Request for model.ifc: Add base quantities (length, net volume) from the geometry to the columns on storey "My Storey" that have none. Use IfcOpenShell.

First a look at what the model holds.

```python
import ifcopenshell
import ifcopenshell.util.element
import ifcopenshell.util.unit

model = ifcopenshell.open("model.ifc")
print(model.schema)
for unit_type in ("LENGTHUNIT", "AREAUNIT", "VOLUMEUNIT"):
    print(unit_type, ifcopenshell.util.unit.calculate_unit_scale(model, unit_type))
storey = next(s for s in model.by_type("IfcBuildingStorey") if s.Name == "My Storey")
columns = [e for e in ifcopenshell.util.element.get_decomposition(storey) if e.is_a("IfcColumn")]
for e in sorted(columns, key=lambda e: e.id()):
    print(e.id(), e.is_a(), e.Name, list(ifcopenshell.util.element.get_psets(e, qtos_only=True)), sep=" | ")
```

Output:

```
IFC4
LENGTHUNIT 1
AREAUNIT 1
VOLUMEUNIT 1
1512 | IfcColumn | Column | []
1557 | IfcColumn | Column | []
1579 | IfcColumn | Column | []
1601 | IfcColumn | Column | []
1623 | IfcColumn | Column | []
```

```python
import ifcopenshell
import ifcopenshell.api.pset
import ifcopenshell.geom
import ifcopenshell.util.element
import ifcopenshell.util.shape
import ifcopenshell.util.unit

model = ifcopenshell.open("model.ifc")
unit_scale = ifcopenshell.util.unit.calculate_unit_scale(model)
volume_scale = ifcopenshell.util.unit.calculate_unit_scale(model, "VOLUMEUNIT")
settings = ifcopenshell.geom.settings()

storey = next(s for s in model.by_type("IfcBuildingStorey") if s.Name == "My Storey")
columns = [e for e in ifcopenshell.util.element.get_decomposition(storey) if e.is_a("IfcColumn")]

for e in sorted(columns, key=lambda e: e.id()):
    if ifcopenshell.util.element.get_psets(e, qtos_only=True, should_inherit=False):
        continue
    # Geometry comes back in metres, in the element's own axes.
    shape = ifcopenshell.geom.create_shape(settings, e)
    values = {
        "Length": ifcopenshell.util.shape.get_z(shape.geometry) / unit_scale,
        "NetVolume": ifcopenshell.util.shape.get_volume(shape.geometry) / volume_scale,
    }
    qto = ifcopenshell.api.pset.add_qto(model, product=e, name="Qto_ColumnBaseQuantities")
    ifcopenshell.api.pset.edit_qto(model, qto=qto, properties=values)
    print(e.id(), {k: round(v, 3) for k, v in values.items()})

model.write("model_updated.ifc")
```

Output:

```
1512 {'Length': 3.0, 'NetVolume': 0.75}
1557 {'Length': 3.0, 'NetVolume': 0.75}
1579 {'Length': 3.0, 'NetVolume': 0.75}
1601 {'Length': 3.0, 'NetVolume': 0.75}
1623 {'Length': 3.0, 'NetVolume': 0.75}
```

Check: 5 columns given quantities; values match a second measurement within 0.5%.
